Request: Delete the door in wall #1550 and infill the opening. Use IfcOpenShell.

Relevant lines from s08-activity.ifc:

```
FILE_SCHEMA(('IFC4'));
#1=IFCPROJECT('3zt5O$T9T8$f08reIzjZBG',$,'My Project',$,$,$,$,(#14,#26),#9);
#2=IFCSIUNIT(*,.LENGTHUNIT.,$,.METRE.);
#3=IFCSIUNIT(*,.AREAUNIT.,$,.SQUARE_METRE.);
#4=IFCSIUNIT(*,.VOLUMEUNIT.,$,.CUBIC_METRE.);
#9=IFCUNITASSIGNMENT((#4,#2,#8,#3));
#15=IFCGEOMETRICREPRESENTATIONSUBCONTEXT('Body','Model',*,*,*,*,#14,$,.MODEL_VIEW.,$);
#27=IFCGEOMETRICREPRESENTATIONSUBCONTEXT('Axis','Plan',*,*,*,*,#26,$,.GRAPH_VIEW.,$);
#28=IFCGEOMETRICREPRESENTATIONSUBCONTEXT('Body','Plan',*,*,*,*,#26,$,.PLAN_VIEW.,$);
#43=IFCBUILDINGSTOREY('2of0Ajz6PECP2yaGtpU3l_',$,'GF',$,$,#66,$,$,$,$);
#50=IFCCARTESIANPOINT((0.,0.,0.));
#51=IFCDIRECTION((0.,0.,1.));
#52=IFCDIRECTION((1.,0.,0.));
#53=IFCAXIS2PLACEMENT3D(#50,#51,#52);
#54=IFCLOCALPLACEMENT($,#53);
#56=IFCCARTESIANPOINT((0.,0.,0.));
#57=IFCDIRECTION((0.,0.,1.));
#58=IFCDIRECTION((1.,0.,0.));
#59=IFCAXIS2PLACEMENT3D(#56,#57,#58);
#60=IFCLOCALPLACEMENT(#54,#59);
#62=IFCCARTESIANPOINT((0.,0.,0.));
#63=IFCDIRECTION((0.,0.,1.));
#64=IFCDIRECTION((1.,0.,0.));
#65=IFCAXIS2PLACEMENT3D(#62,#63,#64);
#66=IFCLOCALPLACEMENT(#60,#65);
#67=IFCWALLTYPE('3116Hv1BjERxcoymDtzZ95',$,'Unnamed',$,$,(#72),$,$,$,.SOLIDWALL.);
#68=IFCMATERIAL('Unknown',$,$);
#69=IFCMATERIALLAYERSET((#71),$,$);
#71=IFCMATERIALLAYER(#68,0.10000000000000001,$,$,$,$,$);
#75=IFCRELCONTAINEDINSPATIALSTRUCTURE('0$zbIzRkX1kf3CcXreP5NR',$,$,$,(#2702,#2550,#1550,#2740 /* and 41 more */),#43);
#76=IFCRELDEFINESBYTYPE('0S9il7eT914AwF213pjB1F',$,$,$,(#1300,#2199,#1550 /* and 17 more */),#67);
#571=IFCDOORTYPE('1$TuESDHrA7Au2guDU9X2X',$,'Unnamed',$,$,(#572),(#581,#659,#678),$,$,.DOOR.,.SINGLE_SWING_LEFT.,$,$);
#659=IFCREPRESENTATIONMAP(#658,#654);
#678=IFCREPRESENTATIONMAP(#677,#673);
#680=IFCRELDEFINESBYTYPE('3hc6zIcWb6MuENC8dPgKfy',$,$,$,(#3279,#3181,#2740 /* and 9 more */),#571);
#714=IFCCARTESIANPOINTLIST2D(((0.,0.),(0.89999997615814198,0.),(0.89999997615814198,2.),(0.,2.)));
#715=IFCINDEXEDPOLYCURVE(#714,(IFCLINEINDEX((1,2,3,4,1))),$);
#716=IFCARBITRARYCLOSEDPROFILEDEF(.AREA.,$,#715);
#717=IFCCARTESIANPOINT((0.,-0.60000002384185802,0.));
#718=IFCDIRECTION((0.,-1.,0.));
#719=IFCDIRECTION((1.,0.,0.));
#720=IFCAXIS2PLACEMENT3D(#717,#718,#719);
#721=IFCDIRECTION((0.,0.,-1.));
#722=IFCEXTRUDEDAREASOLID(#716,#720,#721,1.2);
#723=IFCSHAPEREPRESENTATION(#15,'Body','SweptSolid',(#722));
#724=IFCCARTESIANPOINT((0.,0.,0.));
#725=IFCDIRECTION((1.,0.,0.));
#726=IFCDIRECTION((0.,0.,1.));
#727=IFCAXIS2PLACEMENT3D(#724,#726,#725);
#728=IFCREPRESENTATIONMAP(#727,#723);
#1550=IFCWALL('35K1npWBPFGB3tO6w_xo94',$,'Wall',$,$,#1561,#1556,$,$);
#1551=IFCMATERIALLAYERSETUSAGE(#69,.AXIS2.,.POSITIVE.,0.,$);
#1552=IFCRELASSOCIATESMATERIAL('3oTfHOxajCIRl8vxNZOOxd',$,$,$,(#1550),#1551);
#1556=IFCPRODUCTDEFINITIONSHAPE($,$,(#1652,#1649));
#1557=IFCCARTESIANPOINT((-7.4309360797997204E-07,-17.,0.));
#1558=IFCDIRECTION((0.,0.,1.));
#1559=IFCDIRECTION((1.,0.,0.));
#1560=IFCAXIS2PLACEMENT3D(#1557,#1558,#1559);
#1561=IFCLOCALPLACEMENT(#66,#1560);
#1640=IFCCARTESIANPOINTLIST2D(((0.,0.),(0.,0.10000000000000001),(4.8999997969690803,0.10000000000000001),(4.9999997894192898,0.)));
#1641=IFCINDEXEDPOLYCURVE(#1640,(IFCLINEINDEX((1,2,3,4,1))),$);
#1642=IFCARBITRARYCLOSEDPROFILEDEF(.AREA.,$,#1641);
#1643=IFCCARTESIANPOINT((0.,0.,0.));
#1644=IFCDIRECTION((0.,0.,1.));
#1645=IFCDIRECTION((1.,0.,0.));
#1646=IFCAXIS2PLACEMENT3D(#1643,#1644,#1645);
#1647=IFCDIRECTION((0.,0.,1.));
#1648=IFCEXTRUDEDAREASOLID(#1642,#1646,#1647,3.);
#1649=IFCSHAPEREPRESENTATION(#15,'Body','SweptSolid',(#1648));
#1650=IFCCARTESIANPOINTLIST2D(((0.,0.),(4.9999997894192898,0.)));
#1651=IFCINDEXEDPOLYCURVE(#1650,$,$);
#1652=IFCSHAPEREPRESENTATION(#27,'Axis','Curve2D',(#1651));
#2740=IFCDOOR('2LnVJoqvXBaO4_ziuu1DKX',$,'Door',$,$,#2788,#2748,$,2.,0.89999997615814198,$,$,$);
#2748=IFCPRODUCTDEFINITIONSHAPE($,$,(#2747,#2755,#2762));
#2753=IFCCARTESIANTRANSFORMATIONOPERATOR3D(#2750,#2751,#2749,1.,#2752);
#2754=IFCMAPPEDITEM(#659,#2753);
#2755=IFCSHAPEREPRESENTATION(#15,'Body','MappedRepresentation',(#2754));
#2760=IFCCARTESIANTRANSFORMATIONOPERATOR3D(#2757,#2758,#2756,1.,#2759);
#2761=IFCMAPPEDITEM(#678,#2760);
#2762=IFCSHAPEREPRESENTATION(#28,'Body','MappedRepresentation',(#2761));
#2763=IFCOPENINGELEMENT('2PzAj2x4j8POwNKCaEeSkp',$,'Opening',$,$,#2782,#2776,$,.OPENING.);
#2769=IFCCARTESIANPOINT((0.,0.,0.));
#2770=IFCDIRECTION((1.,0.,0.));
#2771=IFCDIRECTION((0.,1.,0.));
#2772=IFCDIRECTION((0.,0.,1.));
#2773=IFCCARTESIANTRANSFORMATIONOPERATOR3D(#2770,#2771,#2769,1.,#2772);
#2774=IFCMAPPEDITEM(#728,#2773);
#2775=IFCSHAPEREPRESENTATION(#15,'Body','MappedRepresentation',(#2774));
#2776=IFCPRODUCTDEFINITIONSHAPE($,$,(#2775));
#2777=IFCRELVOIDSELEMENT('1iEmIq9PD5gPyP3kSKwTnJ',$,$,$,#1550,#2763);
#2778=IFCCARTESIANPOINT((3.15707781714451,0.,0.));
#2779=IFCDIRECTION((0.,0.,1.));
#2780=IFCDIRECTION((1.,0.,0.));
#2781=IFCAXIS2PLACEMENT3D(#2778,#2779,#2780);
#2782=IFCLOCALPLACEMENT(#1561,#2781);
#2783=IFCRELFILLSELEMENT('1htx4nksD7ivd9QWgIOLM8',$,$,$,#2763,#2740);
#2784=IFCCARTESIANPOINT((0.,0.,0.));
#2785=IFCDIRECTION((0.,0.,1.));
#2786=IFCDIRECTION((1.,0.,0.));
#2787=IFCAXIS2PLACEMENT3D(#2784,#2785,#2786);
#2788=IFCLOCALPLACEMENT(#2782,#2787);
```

```python
import ifcopenshell
import ifcopenshell.api.feature
import ifcopenshell.api.root
import ifcopenshell.geom
import ifcopenshell.util.shape

model = ifcopenshell.open("s08-activity.ifc")
settings = ifcopenshell.geom.settings()


def volume(element):
    """Net volume in cubic metres, openings subtracted."""
    shape = ifcopenshell.geom.create_shape(settings, element)
    return ifcopenshell.util.shape.get_volume(shape.geometry)


door = model.by_guid("2LnVJoqvXBaO4_ziuu1DKX")
opening = door.FillsVoids[0].RelatingOpeningElement
wall = opening.VoidsElements[0].RelatingBuildingElement
before = volume(wall)

ifcopenshell.api.root.remove_product(model, product=door)
ifcopenshell.api.feature.remove_feature(model, feature=opening)

after = volume(wall)

print(f"wall volume {before:.3f} -> {after:.3f} m3")

model.write("s08-activity-out.ifc")
```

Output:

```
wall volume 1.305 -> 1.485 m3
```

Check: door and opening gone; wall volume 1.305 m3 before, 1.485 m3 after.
